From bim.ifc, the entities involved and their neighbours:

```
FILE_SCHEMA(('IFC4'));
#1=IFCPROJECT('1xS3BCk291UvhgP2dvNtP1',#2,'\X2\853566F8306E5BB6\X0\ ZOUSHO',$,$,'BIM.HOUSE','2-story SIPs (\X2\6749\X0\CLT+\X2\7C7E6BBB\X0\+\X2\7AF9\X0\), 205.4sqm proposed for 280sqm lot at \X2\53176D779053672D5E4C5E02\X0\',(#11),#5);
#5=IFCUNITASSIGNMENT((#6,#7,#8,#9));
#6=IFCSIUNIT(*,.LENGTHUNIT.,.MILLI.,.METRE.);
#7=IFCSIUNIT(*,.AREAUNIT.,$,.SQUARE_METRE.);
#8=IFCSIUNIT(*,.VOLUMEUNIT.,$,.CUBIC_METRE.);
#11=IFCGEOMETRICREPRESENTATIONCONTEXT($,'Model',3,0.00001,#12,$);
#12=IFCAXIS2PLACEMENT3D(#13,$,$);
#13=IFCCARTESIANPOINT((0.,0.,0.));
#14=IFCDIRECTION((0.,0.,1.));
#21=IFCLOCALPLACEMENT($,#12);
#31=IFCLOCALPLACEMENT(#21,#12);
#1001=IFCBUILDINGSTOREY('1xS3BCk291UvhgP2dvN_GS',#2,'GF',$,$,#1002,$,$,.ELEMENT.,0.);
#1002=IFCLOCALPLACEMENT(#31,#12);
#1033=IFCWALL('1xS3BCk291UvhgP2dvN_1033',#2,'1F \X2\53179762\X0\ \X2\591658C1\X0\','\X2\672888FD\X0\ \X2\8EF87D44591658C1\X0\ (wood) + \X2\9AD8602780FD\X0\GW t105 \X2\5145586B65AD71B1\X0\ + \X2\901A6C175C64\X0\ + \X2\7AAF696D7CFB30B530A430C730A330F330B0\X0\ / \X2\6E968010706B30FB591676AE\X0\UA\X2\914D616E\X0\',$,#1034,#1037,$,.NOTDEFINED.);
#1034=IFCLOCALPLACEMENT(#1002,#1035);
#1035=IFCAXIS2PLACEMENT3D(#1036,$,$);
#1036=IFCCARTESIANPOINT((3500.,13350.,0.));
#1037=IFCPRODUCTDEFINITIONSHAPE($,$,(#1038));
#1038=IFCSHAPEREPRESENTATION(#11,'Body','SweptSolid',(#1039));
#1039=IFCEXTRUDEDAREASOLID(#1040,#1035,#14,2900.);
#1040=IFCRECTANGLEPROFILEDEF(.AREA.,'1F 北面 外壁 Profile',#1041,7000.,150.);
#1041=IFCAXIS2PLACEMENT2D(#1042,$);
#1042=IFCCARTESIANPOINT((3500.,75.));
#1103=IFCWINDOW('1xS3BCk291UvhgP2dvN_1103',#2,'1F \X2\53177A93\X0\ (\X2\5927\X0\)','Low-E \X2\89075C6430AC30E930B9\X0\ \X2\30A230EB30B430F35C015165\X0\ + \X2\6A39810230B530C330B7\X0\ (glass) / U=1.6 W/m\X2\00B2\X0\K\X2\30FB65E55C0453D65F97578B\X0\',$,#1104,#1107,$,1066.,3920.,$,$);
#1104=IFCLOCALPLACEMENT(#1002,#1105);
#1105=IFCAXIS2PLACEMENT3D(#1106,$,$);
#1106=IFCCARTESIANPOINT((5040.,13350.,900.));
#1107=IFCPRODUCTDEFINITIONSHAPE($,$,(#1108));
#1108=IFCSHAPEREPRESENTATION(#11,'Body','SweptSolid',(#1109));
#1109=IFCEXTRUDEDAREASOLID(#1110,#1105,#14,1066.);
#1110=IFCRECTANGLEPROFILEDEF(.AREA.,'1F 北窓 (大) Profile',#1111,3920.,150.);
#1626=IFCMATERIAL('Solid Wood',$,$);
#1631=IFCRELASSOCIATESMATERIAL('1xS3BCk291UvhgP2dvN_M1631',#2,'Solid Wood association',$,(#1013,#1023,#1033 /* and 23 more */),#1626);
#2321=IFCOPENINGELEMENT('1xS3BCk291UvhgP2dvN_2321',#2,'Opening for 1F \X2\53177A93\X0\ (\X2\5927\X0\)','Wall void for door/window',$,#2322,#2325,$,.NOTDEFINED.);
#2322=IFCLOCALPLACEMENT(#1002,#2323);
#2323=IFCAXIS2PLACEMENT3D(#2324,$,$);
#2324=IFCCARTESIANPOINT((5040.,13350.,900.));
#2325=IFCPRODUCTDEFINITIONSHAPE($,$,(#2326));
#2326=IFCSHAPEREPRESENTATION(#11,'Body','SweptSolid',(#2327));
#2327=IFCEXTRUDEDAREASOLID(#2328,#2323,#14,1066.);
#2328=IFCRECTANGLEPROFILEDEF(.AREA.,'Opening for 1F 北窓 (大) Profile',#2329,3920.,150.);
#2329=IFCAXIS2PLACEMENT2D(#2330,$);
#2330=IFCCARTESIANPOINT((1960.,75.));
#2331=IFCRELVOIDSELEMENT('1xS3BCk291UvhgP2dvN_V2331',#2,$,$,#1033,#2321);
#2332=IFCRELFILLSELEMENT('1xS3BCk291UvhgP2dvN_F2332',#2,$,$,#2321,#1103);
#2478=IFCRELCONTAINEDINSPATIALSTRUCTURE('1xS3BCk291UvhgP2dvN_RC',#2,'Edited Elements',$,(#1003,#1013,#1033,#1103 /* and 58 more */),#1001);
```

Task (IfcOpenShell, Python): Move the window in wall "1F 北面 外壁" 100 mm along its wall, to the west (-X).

```python
import ifcopenshell
import ifcopenshell.api.geometry
import ifcopenshell.util.placement
import ifcopenshell.util.unit

model = ifcopenshell.open("bim.ifc")
unit_scale = ifcopenshell.util.unit.calculate_unit_scale(model)

window = model.by_guid("1xS3BCk291UvhgP2dvN_1103")
opening = window.FillsVoids[0].RelatingOpeningElement
wall = opening.VoidsElements[0].RelatingBuildingElement

wall_matrix = ifcopenshell.util.placement.get_local_placement(wall.ObjectPlacement)
shift = wall_matrix[:3, 0] * -0.1 / unit_scale
before = ifcopenshell.util.placement.get_local_placement(window.ObjectPlacement)[:3, 3].copy()

# The window is not placed relative to its opening, so move both.
for product in (opening, window):
    matrix = ifcopenshell.util.placement.get_local_placement(product.ObjectPlacement)
    matrix[:3, 3] += shift
    ifcopenshell.api.geometry.edit_object_placement(model, product=product, matrix=matrix, is_si=False)

after = ifcopenshell.util.placement.get_local_placement(window.ObjectPlacement)[:3, 3]
print("window moved by", (after - before).round(3) + 0.0)

model.write("bim_rev.ifc")
```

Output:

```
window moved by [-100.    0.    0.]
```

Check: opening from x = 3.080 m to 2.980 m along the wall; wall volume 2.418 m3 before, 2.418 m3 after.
